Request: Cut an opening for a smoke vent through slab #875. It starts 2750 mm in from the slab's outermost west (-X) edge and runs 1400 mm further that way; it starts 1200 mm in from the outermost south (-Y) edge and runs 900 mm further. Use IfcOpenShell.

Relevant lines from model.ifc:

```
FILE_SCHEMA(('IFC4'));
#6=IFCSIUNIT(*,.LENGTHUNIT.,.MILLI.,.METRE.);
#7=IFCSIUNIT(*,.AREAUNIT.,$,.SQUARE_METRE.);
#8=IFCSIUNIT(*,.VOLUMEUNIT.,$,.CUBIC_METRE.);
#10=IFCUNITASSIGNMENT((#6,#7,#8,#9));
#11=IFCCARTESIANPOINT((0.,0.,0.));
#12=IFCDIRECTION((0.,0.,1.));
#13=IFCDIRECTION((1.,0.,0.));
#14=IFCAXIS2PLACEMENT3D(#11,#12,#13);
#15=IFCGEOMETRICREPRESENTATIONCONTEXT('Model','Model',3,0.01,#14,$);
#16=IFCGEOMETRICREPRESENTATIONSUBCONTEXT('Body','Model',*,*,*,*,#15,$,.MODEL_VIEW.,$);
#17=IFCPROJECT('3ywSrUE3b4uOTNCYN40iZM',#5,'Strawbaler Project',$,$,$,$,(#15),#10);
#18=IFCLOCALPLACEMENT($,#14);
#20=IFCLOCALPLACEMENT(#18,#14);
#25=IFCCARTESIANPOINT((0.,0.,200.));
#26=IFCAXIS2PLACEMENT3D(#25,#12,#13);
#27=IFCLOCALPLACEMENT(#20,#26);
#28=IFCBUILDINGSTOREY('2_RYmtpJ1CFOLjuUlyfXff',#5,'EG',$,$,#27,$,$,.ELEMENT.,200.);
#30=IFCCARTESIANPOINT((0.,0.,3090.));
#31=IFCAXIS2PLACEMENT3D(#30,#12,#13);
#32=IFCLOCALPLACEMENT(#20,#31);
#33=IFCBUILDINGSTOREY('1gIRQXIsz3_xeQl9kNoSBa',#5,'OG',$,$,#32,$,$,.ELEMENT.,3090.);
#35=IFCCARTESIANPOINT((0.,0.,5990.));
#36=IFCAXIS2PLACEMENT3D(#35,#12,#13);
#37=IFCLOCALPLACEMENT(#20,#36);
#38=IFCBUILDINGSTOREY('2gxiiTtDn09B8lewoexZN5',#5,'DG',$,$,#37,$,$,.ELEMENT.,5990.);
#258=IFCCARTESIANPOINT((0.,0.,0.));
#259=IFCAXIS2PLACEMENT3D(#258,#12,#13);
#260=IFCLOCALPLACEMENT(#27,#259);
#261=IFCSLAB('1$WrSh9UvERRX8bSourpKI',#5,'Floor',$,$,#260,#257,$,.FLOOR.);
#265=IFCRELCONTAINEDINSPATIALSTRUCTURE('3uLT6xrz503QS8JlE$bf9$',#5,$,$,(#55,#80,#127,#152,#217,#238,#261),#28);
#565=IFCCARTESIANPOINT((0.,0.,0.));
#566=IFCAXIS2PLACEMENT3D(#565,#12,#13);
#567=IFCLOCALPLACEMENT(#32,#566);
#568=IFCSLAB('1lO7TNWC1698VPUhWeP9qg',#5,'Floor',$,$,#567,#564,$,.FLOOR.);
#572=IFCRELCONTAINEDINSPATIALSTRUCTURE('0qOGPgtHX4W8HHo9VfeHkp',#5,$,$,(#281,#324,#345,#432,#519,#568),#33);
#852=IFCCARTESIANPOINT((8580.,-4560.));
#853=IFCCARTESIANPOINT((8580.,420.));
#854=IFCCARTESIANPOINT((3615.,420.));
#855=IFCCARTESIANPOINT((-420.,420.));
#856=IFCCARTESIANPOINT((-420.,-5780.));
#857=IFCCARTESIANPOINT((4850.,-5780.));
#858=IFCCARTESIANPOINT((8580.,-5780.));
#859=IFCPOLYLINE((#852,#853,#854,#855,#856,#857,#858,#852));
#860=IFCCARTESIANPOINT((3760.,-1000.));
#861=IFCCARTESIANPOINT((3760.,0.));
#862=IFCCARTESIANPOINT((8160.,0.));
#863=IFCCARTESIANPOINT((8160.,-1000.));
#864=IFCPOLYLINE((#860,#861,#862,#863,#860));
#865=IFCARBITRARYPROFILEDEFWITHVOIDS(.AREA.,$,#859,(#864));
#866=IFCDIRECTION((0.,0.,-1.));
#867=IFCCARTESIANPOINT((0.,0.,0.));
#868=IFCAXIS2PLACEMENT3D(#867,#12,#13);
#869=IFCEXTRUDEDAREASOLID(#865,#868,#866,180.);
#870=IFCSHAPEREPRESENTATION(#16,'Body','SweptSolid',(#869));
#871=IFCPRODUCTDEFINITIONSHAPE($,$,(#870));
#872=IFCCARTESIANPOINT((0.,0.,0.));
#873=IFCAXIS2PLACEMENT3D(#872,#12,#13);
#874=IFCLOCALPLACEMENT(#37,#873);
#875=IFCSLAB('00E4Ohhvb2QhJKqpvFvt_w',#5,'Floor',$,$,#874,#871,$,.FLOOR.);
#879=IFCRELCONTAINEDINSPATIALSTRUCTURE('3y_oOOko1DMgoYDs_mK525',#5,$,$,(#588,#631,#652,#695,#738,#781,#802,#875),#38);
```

```python
import numpy as np
import ifcopenshell
import ifcopenshell.api.feature
import ifcopenshell.api.geometry
import ifcopenshell.api.root
import ifcopenshell.geom
import ifcopenshell.util.placement
import ifcopenshell.util.representation
import ifcopenshell.util.shape
import ifcopenshell.util.unit

model = ifcopenshell.open("model.ifc")
unit_scale = ifcopenshell.util.unit.calculate_unit_scale(model)
settings = ifcopenshell.geom.settings()


def volume(element):
    """Net volume in cubic metres, openings subtracted."""
    shape = ifcopenshell.geom.create_shape(settings, element)
    return ifcopenshell.util.shape.get_volume(shape.geometry)


slab = model.by_id(875)
before = volume(slab)

# Extent in the slab's own axes, in metres. The edges named are its -X and -Y sides.
slab_shape = ifcopenshell.geom.create_shape(settings, slab)
vertices = ifcopenshell.util.shape.get_vertices(slab_shape.geometry)
x_min, y_min, bottom = vertices.min(axis=0)
top = vertices[:, 2].max()

opening = ifcopenshell.api.root.create_entity(model, ifc_class="IfcOpeningElement", name="Smoke vent opening", predefined_type="OPENING")
context = ifcopenshell.util.representation.get_context(model, "Model", "Body", "MODEL_VIEW")
width, depth = 1.4, 0.9
outline = [(0.0, 0.0), (width, 0.0), (width, depth), (0.0, depth), (0.0, 0.0)]
# Overshoot both faces by 50 mm so the cut is clean.
shape = ifcopenshell.api.geometry.add_slab_representation(
    model, context=context, depth=top - bottom + 0.1, polyline=outline
)
ifcopenshell.api.geometry.assign_representation(model, product=opening, representation=shape)

matrix = ifcopenshell.util.placement.get_local_placement(slab.ObjectPlacement)
matrix[:, 3] = matrix @ np.append(np.array([x_min + 2.75, y_min + 1.2, bottom - 0.05]) / unit_scale, 1.0)
ifcopenshell.api.geometry.edit_object_placement(model, product=opening, matrix=matrix, is_si=False)
ifcopenshell.api.feature.add_feature(model, feature=opening, element=slab)

after = volume(slab)

print(f"slab volume {before:.3f} -> {after:.3f} m3")

model.write("model_updated.ifc")
```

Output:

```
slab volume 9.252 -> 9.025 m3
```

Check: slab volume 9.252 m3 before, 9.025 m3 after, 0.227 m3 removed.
